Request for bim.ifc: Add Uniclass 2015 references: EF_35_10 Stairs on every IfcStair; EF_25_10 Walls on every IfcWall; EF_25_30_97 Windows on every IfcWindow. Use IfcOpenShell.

First a look at what the model holds.

```python
import ifcopenshell

model = ifcopenshell.open("bim.ifc")
print(model.schema)
print("classifications:", [c.Name for c in model.by_type("IfcClassification")])
for ifc_class in ("IfcDoor", "IfcRoof", "IfcStair", "IfcWall", "IfcWindow"):
    print(ifc_class, len(model.by_type(ifc_class)))
```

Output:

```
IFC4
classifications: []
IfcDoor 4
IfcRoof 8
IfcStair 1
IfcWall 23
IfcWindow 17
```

```python
import ifcopenshell
import ifcopenshell.api.classification

model = ifcopenshell.open("bim.ifc")

system = ifcopenshell.api.classification.add_classification(model, classification="Uniclass 2015")

codes = {
    "IfcStair": ("EF_35_10", "Stairs"),
    "IfcWall": ("EF_25_10", "Walls"),
    "IfcWindow": ("EF_25_30_97", "Windows"),
}
for ifc_class, (code, name) in codes.items():
    products = model.by_type(ifc_class)
    ifcopenshell.api.classification.add_reference(
        model, products=products, classification=system, identification=code, name=name
    )
    print(code, len(products))

model.write("bim-out.ifc")
```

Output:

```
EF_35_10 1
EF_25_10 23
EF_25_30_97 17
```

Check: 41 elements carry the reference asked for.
